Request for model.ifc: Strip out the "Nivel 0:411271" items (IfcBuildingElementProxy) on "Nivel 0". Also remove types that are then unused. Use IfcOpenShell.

First a look at what the model holds.

```python
import ifcopenshell
import ifcopenshell.util.element

model = ifcopenshell.open("model.ifc")
print(model.schema)
storey = next(s for s in model.by_type("IfcBuildingStorey") if s.Name == "Nivel 0")
proxies = [e for e in ifcopenshell.util.element.get_decomposition(storey) if e.is_a("IfcBuildingElementProxy")]
seen = {}
for e in proxies:
    element_type = ifcopenshell.util.element.get_type(e)
    name = element_type.Name if element_type not in (None, e) else None
    seen[name] = seen.get(name, 0) + 1
for name, count in sorted(seen.items(), key=str):
    print(count, "x", name)
```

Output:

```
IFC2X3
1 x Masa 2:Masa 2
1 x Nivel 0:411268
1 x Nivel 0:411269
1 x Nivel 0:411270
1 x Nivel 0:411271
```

```python
import ifcopenshell
import ifcopenshell.api.root
import ifcopenshell.util.element

model = ifcopenshell.open("model.ifc")

storey = next(s for s in model.by_type("IfcBuildingStorey") if s.Name == "Nivel 0")
proxies = [e for e in ifcopenshell.util.element.get_decomposition(storey) if e.is_a("IfcBuildingElementProxy")]
targets = [e for e in proxies if (t := ifcopenshell.util.element.get_type(e)) not in (None, e) and t.Name == "Nivel 0:411271"]
types = {ifcopenshell.util.element.get_type(e) for e in targets} - {None, *targets}

for e in targets:
    ifcopenshell.api.root.remove_product(model, product=e)
print(len(targets), "removed")

unused = [t for t in types if not ifcopenshell.util.element.get_types(t)]
for t in unused:
    ifcopenshell.api.root.remove_product(model, product=t)
print(len(unused), "unused types removed")

model.write("model_updated.ifc")
```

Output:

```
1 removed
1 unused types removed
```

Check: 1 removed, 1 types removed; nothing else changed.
